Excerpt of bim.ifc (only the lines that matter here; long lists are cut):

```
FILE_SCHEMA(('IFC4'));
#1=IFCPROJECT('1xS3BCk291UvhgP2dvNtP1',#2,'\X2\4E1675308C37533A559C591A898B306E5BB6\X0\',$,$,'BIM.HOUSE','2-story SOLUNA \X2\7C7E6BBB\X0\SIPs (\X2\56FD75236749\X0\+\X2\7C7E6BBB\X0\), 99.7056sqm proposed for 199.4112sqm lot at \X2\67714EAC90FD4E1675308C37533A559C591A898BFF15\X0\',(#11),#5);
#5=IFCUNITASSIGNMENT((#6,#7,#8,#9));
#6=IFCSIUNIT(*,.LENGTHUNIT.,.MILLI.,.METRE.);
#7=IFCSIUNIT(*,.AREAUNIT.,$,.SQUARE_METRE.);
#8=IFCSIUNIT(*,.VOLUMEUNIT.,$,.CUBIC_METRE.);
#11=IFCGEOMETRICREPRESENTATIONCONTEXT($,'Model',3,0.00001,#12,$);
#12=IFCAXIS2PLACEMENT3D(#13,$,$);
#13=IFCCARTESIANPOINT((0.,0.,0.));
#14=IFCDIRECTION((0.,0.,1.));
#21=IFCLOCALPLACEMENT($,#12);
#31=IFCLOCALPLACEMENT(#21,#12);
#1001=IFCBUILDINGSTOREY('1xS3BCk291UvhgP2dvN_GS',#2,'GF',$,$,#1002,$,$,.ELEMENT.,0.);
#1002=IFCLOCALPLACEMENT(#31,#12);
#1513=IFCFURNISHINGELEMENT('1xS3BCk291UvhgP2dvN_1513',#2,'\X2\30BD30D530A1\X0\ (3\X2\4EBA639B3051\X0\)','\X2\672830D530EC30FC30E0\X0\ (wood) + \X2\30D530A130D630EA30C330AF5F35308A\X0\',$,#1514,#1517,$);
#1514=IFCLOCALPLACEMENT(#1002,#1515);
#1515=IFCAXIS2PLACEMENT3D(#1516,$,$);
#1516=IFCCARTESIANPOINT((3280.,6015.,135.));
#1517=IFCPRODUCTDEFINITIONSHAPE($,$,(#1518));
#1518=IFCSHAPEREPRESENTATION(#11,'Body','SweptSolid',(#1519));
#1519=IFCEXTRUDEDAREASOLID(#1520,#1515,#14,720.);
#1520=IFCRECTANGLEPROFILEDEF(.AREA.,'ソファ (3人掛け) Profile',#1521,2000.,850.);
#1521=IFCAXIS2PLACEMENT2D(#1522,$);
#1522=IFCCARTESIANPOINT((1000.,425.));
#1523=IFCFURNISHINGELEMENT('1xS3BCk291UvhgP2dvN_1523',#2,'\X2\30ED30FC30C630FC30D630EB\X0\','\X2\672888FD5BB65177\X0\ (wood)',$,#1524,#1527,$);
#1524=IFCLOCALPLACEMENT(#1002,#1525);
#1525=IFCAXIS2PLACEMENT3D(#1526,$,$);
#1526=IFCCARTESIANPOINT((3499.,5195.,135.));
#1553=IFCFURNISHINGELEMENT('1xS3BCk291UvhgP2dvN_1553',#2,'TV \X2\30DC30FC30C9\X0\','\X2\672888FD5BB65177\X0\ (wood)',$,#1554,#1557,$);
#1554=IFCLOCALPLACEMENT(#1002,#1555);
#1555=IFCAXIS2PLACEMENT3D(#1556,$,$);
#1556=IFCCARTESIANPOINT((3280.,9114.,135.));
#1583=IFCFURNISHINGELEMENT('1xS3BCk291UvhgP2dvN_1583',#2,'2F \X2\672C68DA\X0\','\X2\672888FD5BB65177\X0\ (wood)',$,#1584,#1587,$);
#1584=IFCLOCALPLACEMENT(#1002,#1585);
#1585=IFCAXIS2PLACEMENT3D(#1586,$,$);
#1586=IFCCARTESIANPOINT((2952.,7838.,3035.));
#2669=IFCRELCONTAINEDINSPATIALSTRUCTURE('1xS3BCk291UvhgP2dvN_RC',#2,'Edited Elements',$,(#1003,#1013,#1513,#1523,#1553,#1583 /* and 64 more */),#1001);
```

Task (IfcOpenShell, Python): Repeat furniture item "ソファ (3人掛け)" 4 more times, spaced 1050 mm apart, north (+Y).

```python
import numpy as np
import ifcopenshell
import ifcopenshell.api.geometry
import ifcopenshell.api.root
import ifcopenshell.util.element
import ifcopenshell.util.placement
import ifcopenshell.util.unit

model = ifcopenshell.open("bim.ifc")
unit_scale = ifcopenshell.util.unit.calculate_unit_scale(model)


def reuse_history(source, copy):
    """copy_class also copies each property set's owner history, people and application; keep the originals."""
    for rel in copy.IsDefinedBy:
        if rel.is_a("IfcRelDefinesByProperties") and (history := rel.RelatingPropertyDefinition.OwnerHistory):
            rel.RelatingPropertyDefinition.OwnerHistory = source.OwnerHistory
            ifcopenshell.util.element.remove_deep2(model, history)


source = model.by_id(1513)
base = ifcopenshell.util.placement.get_local_placement(source.ObjectPlacement)
step = np.array([0.0, 1.0, 0.0]) * 1.05 / unit_scale

for i in range(1, 5):
    copy = ifcopenshell.api.root.copy_class(model, product=source)
    copy.Representation = ifcopenshell.util.element.copy_deep(
        model, source.Representation, exclude=["IfcGeometricRepresentationContext", "IfcRepresentationMap"]
    )
    reuse_history(source, copy)
    matrix = base.copy()
    matrix[:3, 3] += i * step
    print("added at", matrix[:3, 3].round(3) + 0.0)
    ifcopenshell.api.geometry.edit_object_placement(model, product=copy, matrix=matrix, is_si=False)

model.write("bim_updated.ifc")
```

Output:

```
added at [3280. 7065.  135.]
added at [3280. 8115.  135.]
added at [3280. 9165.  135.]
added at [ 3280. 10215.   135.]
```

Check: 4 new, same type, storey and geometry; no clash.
